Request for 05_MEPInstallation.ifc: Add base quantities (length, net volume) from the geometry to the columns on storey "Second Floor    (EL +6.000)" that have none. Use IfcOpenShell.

First a look at what the model holds.

```python
import ifcopenshell
import ifcopenshell.util.element
import ifcopenshell.util.unit

model = ifcopenshell.open("05_MEPInstallation.ifc")
print(model.schema)
for unit_type in ("LENGTHUNIT", "AREAUNIT", "VOLUMEUNIT"):
    print(unit_type, ifcopenshell.util.unit.calculate_unit_scale(model, unit_type))
storey = next(s for s in model.by_type("IfcBuildingStorey") if s.Name == "Second Floor    (EL +6.000)")
columns = [e for e in ifcopenshell.util.element.get_decomposition(storey) if e.is_a("IfcColumn")]
for e in sorted(columns, key=lambda e: e.id()):
    print(e.id(), e.is_a(), e.Name, list(ifcopenshell.util.element.get_psets(e, qtos_only=True)), sep=" | ")
```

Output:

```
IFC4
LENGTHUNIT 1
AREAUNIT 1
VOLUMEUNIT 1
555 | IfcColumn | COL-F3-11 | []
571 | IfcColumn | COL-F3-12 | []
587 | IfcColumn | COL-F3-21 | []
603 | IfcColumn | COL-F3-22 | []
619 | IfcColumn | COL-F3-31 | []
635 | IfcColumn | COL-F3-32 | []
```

```python
import ifcopenshell
import ifcopenshell.api.pset
import ifcopenshell.geom
import ifcopenshell.util.element
import ifcopenshell.util.shape
import ifcopenshell.util.unit

model = ifcopenshell.open("05_MEPInstallation.ifc")
unit_scale = ifcopenshell.util.unit.calculate_unit_scale(model)
volume_scale = ifcopenshell.util.unit.calculate_unit_scale(model, "VOLUMEUNIT")
settings = ifcopenshell.geom.settings()

storey = next(s for s in model.by_type("IfcBuildingStorey") if s.Name == "Second Floor    (EL +6.000)")
columns = [e for e in ifcopenshell.util.element.get_decomposition(storey) if e.is_a("IfcColumn")]

for e in sorted(columns, key=lambda e: e.id()):
    if ifcopenshell.util.element.get_psets(e, qtos_only=True, should_inherit=False):
        continue
    # Geometry comes back in metres, in the element's own axes.
    shape = ifcopenshell.geom.create_shape(settings, e)
    values = {
        "Length": ifcopenshell.util.shape.get_z(shape.geometry) / unit_scale,
        "NetVolume": ifcopenshell.util.shape.get_volume(shape.geometry) / volume_scale,
    }
    qto = ifcopenshell.api.pset.add_qto(model, product=e, name="Qto_ColumnBaseQuantities")
    ifcopenshell.api.pset.edit_qto(model, qto=qto, properties=values)
    print(e.id(), {k: round(v, 3) for k, v in values.items()})

model.write("05_MEPInstallation_v2.ifc")
```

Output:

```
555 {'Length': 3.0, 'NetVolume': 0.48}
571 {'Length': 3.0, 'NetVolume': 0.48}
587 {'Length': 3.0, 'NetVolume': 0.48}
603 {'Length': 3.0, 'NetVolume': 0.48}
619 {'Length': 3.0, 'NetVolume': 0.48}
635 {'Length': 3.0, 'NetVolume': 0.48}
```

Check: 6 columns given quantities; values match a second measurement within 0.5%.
